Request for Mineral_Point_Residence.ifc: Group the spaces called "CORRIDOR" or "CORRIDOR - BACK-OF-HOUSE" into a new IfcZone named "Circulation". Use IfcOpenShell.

First a look at what the model holds.

```python
import ifcopenshell

model = ifcopenshell.open("Mineral_Point_Residence.ifc")
print(model.schema)
seen = {}
for space in model.by_type("IfcSpace"):
    seen[space.LongName] = seen.get(space.LongName, 0) + 1
for name, count in sorted(seen.items(), key=str):
    print(count, "x", name)
print("zones:", [z.Name for z in model.by_type("IfcZone")][:20])
```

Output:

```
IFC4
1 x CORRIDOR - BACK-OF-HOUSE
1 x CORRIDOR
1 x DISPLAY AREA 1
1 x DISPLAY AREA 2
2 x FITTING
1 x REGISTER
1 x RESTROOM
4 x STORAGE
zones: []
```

```python
import ifcopenshell
import ifcopenshell.api.group
import ifcopenshell.api.root

model = ifcopenshell.open("Mineral_Point_Residence.ifc")

names = {"CORRIDOR", "CORRIDOR - BACK-OF-HOUSE"}
spaces = [s for s in model.by_type("IfcSpace") if s.LongName in names]

zone = ifcopenshell.api.root.create_entity(model, ifc_class="IfcZone", name="Circulation")
ifcopenshell.api.group.assign_group(model, products=spaces, group=zone)
print(len(spaces), "spaces in", zone.Name)

model.write("Mineral_Point_Residence_rev.ifc")
```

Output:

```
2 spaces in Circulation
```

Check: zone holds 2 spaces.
